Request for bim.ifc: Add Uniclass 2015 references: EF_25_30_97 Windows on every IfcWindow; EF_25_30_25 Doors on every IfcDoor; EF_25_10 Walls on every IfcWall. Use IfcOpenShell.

First a look at what the model holds.

```python
import ifcopenshell

model = ifcopenshell.open("bim.ifc")
print(model.schema)
print("classifications:", [c.Name for c in model.by_type("IfcClassification")])
for ifc_class in ("IfcDoor", "IfcRoof", "IfcStair", "IfcWall", "IfcWindow"):
    print(ifc_class, len(model.by_type(ifc_class)))
```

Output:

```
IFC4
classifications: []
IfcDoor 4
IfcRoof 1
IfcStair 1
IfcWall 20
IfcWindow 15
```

```python
import ifcopenshell
import ifcopenshell.api.classification

model = ifcopenshell.open("bim.ifc")

system = ifcopenshell.api.classification.add_classification(model, classification="Uniclass 2015")

codes = {
    "IfcWindow": ("EF_25_30_97", "Windows"),
    "IfcDoor": ("EF_25_30_25", "Doors"),
    "IfcWall": ("EF_25_10", "Walls"),
}
for ifc_class, (code, name) in codes.items():
    products = model.by_type(ifc_class)
    ifcopenshell.api.classification.add_reference(
        model, products=products, classification=system, identification=code, name=name
    )
    print(code, len(products))

model.write("bim-out.ifc")
```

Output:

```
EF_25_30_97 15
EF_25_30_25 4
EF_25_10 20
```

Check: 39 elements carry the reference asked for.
